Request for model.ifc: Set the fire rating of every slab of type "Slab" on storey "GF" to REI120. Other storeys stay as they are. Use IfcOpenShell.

First a look at what the model holds.

```python
import ifcopenshell
import ifcopenshell.util.element

model = ifcopenshell.open("model.ifc")
print(model.schema)
storey = next(s for s in model.by_type("IfcBuildingStorey") if s.Name == "GF")
slabs = [e for e in ifcopenshell.util.element.get_decomposition(storey) if e.is_a("IfcSlab")]
seen = {}
for e in slabs:
    element_type = ifcopenshell.util.element.get_type(e)
    key = (element_type.Name if element_type != e and element_type else None, ifcopenshell.util.element.get_pset(e, "Pset_SlabCommon", "FireRating"))
    seen[key] = seen.get(key, 0) + 1
for (name, value), count in sorted(seen.items(), key=str):
    print(count, "x", name, "|", value)
```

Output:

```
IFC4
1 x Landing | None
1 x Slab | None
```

```python
import ifcopenshell
import ifcopenshell.api.pset
import ifcopenshell.util.element

model = ifcopenshell.open("model.ifc")

storey = next(s for s in model.by_type("IfcBuildingStorey") if s.Name == "GF")
slabs = [e for e in ifcopenshell.util.element.get_decomposition(storey) if e.is_a("IfcSlab")]

count = 0
for e in slabs:
    element_type = ifcopenshell.util.element.get_type(e)
    if element_type in (None, e) or element_type.Name != "Slab":
        continue
    # add_pset returns the element's existing set when there is one.
    pset = ifcopenshell.api.pset.add_pset(model, product=e, name="Pset_SlabCommon")
    ifcopenshell.api.pset.edit_pset(model, pset=pset, properties={"FireRating": "REI120"})
    count += 1

print(count, "slabs updated")

model.write("model_rev.ifc")
```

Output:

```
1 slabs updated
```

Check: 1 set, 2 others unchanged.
